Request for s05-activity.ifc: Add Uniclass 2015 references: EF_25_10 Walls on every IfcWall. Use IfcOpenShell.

First a look at what the model holds.

```python
import ifcopenshell

model = ifcopenshell.open("s05-activity.ifc")
print(model.schema)
print("classifications:", [c.Name for c in model.by_type("IfcClassification")])
for ifc_class in ("IfcDoor", "IfcRoof", "IfcStair", "IfcWall", "IfcWindow"):
    print(ifc_class, len(model.by_type(ifc_class)))
```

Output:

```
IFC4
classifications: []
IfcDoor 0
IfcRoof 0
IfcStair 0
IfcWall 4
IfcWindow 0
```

```python
import ifcopenshell
import ifcopenshell.api.classification

model = ifcopenshell.open("s05-activity.ifc")

system = ifcopenshell.api.classification.add_classification(model, classification="Uniclass 2015")

codes = {
    "IfcWall": ("EF_25_10", "Walls"),
}
for ifc_class, (code, name) in codes.items():
    products = model.by_type(ifc_class)
    ifcopenshell.api.classification.add_reference(
        model, products=products, classification=system, identification=code, name=name
    )
    print(code, len(products))

model.write("s05-activity_updated.ifc")
```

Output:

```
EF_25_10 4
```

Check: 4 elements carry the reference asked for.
